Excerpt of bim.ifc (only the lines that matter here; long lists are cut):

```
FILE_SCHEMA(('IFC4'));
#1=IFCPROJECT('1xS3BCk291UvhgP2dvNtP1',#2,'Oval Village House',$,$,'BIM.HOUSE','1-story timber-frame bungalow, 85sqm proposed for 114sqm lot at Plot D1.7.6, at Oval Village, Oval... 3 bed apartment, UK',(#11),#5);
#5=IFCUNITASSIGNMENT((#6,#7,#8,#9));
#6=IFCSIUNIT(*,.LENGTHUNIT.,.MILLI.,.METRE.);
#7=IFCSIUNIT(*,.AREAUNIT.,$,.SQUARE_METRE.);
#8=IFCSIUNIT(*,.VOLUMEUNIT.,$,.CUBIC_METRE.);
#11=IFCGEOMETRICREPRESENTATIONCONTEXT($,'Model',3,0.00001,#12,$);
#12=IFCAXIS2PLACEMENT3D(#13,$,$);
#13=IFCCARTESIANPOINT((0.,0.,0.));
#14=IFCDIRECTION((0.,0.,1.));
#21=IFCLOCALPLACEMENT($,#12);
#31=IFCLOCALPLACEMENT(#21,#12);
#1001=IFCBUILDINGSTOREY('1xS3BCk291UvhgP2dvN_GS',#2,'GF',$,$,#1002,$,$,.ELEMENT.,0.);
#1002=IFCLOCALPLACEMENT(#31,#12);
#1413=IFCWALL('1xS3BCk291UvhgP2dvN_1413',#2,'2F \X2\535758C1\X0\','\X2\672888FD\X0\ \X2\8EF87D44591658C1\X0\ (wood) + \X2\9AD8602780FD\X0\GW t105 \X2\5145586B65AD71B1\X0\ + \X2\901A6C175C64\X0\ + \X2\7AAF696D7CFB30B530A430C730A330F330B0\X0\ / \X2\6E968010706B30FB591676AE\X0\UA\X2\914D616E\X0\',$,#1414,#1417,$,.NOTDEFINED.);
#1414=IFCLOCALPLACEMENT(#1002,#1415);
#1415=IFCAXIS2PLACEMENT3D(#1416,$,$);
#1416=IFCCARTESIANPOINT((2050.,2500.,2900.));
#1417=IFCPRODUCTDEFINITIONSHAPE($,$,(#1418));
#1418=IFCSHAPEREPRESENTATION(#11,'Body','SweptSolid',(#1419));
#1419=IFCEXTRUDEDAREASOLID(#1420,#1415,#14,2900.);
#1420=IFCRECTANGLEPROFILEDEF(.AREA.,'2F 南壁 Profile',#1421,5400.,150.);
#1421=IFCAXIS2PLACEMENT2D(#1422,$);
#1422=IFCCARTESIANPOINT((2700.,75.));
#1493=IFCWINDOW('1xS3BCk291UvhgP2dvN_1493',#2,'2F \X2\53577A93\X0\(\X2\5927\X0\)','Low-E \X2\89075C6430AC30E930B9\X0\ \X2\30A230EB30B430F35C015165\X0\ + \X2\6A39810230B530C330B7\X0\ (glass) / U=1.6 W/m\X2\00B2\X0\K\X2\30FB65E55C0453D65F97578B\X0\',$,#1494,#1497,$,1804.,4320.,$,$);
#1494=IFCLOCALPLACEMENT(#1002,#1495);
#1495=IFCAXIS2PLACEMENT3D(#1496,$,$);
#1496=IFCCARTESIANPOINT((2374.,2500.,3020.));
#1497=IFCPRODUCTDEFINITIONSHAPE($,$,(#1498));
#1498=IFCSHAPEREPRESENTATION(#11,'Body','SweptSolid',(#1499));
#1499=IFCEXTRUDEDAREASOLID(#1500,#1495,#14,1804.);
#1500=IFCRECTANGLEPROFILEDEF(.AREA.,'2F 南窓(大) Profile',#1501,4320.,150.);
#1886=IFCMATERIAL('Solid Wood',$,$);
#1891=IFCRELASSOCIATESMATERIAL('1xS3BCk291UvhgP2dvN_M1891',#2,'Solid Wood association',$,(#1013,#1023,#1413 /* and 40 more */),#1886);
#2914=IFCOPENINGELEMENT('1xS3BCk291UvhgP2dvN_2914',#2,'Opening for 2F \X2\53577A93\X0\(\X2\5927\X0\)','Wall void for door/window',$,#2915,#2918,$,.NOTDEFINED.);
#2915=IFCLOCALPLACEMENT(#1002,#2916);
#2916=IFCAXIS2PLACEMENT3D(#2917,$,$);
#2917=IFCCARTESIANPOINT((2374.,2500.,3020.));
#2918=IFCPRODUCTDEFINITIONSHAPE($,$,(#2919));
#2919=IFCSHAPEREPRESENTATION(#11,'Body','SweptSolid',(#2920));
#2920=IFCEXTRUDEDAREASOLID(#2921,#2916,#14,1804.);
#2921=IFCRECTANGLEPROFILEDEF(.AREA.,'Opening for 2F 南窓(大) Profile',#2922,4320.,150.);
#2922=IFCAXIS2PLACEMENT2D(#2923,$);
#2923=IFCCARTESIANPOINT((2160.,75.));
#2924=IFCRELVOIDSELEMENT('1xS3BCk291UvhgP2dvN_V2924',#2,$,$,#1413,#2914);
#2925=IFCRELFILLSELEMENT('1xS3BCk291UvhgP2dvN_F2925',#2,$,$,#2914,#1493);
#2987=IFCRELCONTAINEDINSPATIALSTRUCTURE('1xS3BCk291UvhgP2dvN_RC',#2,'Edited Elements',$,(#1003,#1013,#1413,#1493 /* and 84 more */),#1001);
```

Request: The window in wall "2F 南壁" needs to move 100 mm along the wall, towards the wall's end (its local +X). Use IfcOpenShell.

```python
import ifcopenshell
import ifcopenshell.api.geometry
import ifcopenshell.util.placement
import ifcopenshell.util.unit

model = ifcopenshell.open("bim.ifc")
unit_scale = ifcopenshell.util.unit.calculate_unit_scale(model)

window = model.by_id(1493)
opening = window.FillsVoids[0].RelatingOpeningElement
wall = opening.VoidsElements[0].RelatingBuildingElement

wall_matrix = ifcopenshell.util.placement.get_local_placement(wall.ObjectPlacement)
shift = wall_matrix[:3, 0] * 0.1 / unit_scale
before = ifcopenshell.util.placement.get_local_placement(window.ObjectPlacement)[:3, 3].copy()

# The window is not placed relative to its opening, so move both.
for product in (opening, window):
    matrix = ifcopenshell.util.placement.get_local_placement(product.ObjectPlacement)
    matrix[:3, 3] += shift
    ifcopenshell.api.geometry.edit_object_placement(model, product=product, matrix=matrix, is_si=False)

after = ifcopenshell.util.placement.get_local_placement(window.ObjectPlacement)[:3, 3]
print("window moved by", (after - before).round(3) + 0.0)

model.write("bim_v2.ifc")
```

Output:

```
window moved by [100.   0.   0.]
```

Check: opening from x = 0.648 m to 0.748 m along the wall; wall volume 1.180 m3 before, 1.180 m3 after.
